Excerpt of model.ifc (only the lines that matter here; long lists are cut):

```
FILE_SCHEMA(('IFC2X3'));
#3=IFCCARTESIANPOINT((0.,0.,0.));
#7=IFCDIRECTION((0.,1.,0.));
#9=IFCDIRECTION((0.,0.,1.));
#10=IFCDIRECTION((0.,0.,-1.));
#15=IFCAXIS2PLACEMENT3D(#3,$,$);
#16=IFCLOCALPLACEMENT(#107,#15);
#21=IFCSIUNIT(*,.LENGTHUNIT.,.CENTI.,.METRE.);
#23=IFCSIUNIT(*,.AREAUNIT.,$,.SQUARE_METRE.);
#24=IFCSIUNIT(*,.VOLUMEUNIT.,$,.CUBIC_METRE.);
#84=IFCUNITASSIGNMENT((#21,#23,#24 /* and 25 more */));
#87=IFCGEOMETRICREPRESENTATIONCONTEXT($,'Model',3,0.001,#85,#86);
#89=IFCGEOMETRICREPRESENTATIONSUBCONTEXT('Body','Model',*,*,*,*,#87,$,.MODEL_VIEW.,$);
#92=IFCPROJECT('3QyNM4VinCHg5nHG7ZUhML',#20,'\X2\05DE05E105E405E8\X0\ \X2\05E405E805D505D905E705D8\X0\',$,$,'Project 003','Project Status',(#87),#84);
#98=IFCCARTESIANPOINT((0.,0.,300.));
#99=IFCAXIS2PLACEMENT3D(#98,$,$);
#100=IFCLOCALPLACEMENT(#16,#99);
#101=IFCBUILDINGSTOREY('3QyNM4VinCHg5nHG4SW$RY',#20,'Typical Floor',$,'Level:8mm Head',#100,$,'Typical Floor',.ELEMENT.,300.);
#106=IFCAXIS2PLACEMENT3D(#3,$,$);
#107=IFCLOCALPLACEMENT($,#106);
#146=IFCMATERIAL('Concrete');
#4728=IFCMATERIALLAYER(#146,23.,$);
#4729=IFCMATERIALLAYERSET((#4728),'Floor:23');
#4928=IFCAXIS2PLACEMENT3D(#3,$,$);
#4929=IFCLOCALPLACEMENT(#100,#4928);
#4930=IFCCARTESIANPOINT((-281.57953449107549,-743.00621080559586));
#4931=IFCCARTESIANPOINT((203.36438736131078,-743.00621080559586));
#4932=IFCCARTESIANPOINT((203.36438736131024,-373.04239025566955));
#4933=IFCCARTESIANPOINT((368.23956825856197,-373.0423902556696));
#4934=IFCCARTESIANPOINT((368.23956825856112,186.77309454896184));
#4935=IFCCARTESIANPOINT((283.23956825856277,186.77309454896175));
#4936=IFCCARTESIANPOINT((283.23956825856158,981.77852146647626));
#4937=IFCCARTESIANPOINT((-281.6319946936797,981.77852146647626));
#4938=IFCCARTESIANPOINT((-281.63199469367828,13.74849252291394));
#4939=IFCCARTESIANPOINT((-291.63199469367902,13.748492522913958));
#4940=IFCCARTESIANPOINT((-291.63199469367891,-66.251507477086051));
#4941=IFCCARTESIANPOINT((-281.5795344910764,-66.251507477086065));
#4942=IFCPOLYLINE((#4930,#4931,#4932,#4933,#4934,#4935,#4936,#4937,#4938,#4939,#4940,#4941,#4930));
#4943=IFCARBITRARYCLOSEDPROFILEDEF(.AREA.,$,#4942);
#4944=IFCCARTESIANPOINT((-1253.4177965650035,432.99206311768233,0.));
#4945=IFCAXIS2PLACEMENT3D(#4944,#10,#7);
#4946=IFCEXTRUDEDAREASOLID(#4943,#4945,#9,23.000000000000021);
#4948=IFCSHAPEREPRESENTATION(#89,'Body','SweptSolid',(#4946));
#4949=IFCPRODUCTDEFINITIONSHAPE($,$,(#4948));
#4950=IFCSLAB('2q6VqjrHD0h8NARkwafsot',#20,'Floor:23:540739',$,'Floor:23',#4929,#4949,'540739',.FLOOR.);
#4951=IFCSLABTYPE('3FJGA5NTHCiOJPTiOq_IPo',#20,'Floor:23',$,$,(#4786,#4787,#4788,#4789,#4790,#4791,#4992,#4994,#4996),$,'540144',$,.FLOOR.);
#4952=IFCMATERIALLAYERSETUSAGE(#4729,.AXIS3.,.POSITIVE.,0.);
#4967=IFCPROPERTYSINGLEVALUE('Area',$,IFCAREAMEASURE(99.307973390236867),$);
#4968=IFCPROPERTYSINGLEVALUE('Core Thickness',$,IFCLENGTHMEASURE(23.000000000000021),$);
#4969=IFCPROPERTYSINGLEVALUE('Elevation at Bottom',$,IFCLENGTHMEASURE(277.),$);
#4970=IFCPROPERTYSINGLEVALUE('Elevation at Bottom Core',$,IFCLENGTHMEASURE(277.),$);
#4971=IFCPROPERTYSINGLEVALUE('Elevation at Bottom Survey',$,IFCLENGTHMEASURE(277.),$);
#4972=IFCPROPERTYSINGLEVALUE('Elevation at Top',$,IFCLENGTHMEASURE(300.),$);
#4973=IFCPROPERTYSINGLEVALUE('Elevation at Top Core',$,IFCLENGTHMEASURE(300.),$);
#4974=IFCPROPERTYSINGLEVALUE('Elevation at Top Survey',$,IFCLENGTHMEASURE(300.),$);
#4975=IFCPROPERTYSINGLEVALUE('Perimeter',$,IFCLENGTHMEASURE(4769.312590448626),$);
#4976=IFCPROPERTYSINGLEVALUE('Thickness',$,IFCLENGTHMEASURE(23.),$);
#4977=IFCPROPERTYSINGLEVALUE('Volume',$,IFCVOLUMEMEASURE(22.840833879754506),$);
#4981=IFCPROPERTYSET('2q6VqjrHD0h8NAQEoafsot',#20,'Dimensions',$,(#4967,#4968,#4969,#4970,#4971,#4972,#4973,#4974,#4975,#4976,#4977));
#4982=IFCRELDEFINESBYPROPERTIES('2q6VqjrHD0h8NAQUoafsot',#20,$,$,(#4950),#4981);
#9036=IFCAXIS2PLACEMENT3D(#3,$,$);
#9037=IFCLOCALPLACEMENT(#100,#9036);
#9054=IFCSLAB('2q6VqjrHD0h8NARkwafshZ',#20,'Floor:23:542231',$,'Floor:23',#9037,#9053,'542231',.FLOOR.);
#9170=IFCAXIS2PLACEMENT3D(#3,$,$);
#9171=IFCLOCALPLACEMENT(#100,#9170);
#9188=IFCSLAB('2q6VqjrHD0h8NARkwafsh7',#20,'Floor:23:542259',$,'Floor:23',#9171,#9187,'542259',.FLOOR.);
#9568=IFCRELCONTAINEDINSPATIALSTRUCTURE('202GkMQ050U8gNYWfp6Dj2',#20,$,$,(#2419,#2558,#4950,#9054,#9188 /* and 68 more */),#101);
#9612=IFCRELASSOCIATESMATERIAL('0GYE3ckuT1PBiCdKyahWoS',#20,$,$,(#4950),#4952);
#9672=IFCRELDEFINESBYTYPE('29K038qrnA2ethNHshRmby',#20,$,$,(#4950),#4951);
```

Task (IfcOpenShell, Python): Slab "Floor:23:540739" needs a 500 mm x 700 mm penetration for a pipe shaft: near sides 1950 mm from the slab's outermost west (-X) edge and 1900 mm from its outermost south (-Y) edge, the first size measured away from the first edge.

```python
import numpy as np
import ifcopenshell
import ifcopenshell.api.feature
import ifcopenshell.api.geometry
import ifcopenshell.api.pset
import ifcopenshell.api.root
import ifcopenshell.geom
import ifcopenshell.util.element
import ifcopenshell.util.placement
import ifcopenshell.util.representation
import ifcopenshell.util.shape
import ifcopenshell.util.unit

model = ifcopenshell.open("model.ifc")
unit_scale = ifcopenshell.util.unit.calculate_unit_scale(model)
area_scale = ifcopenshell.util.unit.calculate_unit_scale(model, "AREAUNIT")
volume_scale = ifcopenshell.util.unit.calculate_unit_scale(model, "VOLUMEUNIT")
settings = ifcopenshell.geom.settings()


def volume(element):
    """Net volume in cubic metres, openings subtracted."""
    shape = ifcopenshell.geom.create_shape(settings, element)
    return ifcopenshell.util.shape.get_volume(shape.geometry)


slab = model.by_guid("2q6VqjrHD0h8NARkwafsot")
before = volume(slab)

# Extent in the slab's own axes, in metres. The edges named are its -X and -Y sides.
slab_shape = ifcopenshell.geom.create_shape(settings, slab)
vertices = ifcopenshell.util.shape.get_vertices(slab_shape.geometry)
x_min, y_min, bottom = vertices.min(axis=0)
top = vertices[:, 2].max()

opening = ifcopenshell.api.root.create_entity(model, ifc_class="IfcOpeningElement", name="Pipe shaft opening")
context = ifcopenshell.util.representation.get_context(model, "Model", "Body", "MODEL_VIEW")
width, depth = 0.5, 0.7
outline = [(0.0, 0.0), (width, 0.0), (width, depth), (0.0, depth), (0.0, 0.0)]
# Overshoot both faces by 50 mm so the cut is clean.
shape = ifcopenshell.api.geometry.add_slab_representation(
    model, context=context, depth=top - bottom + 0.1, polyline=outline
)
ifcopenshell.api.geometry.assign_representation(model, product=opening, representation=shape)

matrix = ifcopenshell.util.placement.get_local_placement(slab.ObjectPlacement)
matrix[:, 3] = matrix @ np.append(np.array([x_min + 1.95, y_min + 1.9, bottom - 0.05]) / unit_scale, 1.0)
ifcopenshell.api.geometry.edit_object_placement(model, product=opening, matrix=matrix, is_si=False)
ifcopenshell.api.feature.add_feature(model, feature=opening, element=slab)

after = volume(slab)

# Update the slab's stored quantities.
pset = model.by_id(ifcopenshell.util.element.get_pset(slab, "Dimensions", should_inherit=False)["id"])
ifcopenshell.api.pset.edit_pset(model, pset=pset, properties={
    "Area": model.create_entity("IfcAreaMeasure", after / (top - bottom) / area_scale),
    "Volume": model.create_entity("IfcVolumeMeasure", after / volume_scale),
})

print(f"slab volume {before:.3f} -> {after:.3f} m3")

model.write("model_rev.ifc")
```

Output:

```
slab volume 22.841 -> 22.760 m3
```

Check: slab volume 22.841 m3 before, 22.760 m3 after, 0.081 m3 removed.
